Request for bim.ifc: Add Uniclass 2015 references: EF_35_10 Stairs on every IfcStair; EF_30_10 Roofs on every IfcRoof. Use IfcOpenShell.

First a look at what the model holds.

```python
import ifcopenshell

model = ifcopenshell.open("bim.ifc")
print(model.schema)
print("classifications:", [c.Name for c in model.by_type("IfcClassification")])
for ifc_class in ("IfcDoor", "IfcRoof", "IfcStair", "IfcWall", "IfcWindow"):
    print(ifc_class, len(model.by_type(ifc_class)))
```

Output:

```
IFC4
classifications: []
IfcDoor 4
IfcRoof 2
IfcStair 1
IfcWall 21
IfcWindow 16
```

```python
import ifcopenshell
import ifcopenshell.api.classification

model = ifcopenshell.open("bim.ifc")

system = ifcopenshell.api.classification.add_classification(model, classification="Uniclass 2015")

codes = {
    "IfcStair": ("EF_35_10", "Stairs"),
    "IfcRoof": ("EF_30_10", "Roofs"),
}
for ifc_class, (code, name) in codes.items():
    products = model.by_type(ifc_class)
    ifcopenshell.api.classification.add_reference(
        model, products=products, classification=system, identification=code, name=name
    )
    print(code, len(products))

model.write("bim_edited.ifc")
```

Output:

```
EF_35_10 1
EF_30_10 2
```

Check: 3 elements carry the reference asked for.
